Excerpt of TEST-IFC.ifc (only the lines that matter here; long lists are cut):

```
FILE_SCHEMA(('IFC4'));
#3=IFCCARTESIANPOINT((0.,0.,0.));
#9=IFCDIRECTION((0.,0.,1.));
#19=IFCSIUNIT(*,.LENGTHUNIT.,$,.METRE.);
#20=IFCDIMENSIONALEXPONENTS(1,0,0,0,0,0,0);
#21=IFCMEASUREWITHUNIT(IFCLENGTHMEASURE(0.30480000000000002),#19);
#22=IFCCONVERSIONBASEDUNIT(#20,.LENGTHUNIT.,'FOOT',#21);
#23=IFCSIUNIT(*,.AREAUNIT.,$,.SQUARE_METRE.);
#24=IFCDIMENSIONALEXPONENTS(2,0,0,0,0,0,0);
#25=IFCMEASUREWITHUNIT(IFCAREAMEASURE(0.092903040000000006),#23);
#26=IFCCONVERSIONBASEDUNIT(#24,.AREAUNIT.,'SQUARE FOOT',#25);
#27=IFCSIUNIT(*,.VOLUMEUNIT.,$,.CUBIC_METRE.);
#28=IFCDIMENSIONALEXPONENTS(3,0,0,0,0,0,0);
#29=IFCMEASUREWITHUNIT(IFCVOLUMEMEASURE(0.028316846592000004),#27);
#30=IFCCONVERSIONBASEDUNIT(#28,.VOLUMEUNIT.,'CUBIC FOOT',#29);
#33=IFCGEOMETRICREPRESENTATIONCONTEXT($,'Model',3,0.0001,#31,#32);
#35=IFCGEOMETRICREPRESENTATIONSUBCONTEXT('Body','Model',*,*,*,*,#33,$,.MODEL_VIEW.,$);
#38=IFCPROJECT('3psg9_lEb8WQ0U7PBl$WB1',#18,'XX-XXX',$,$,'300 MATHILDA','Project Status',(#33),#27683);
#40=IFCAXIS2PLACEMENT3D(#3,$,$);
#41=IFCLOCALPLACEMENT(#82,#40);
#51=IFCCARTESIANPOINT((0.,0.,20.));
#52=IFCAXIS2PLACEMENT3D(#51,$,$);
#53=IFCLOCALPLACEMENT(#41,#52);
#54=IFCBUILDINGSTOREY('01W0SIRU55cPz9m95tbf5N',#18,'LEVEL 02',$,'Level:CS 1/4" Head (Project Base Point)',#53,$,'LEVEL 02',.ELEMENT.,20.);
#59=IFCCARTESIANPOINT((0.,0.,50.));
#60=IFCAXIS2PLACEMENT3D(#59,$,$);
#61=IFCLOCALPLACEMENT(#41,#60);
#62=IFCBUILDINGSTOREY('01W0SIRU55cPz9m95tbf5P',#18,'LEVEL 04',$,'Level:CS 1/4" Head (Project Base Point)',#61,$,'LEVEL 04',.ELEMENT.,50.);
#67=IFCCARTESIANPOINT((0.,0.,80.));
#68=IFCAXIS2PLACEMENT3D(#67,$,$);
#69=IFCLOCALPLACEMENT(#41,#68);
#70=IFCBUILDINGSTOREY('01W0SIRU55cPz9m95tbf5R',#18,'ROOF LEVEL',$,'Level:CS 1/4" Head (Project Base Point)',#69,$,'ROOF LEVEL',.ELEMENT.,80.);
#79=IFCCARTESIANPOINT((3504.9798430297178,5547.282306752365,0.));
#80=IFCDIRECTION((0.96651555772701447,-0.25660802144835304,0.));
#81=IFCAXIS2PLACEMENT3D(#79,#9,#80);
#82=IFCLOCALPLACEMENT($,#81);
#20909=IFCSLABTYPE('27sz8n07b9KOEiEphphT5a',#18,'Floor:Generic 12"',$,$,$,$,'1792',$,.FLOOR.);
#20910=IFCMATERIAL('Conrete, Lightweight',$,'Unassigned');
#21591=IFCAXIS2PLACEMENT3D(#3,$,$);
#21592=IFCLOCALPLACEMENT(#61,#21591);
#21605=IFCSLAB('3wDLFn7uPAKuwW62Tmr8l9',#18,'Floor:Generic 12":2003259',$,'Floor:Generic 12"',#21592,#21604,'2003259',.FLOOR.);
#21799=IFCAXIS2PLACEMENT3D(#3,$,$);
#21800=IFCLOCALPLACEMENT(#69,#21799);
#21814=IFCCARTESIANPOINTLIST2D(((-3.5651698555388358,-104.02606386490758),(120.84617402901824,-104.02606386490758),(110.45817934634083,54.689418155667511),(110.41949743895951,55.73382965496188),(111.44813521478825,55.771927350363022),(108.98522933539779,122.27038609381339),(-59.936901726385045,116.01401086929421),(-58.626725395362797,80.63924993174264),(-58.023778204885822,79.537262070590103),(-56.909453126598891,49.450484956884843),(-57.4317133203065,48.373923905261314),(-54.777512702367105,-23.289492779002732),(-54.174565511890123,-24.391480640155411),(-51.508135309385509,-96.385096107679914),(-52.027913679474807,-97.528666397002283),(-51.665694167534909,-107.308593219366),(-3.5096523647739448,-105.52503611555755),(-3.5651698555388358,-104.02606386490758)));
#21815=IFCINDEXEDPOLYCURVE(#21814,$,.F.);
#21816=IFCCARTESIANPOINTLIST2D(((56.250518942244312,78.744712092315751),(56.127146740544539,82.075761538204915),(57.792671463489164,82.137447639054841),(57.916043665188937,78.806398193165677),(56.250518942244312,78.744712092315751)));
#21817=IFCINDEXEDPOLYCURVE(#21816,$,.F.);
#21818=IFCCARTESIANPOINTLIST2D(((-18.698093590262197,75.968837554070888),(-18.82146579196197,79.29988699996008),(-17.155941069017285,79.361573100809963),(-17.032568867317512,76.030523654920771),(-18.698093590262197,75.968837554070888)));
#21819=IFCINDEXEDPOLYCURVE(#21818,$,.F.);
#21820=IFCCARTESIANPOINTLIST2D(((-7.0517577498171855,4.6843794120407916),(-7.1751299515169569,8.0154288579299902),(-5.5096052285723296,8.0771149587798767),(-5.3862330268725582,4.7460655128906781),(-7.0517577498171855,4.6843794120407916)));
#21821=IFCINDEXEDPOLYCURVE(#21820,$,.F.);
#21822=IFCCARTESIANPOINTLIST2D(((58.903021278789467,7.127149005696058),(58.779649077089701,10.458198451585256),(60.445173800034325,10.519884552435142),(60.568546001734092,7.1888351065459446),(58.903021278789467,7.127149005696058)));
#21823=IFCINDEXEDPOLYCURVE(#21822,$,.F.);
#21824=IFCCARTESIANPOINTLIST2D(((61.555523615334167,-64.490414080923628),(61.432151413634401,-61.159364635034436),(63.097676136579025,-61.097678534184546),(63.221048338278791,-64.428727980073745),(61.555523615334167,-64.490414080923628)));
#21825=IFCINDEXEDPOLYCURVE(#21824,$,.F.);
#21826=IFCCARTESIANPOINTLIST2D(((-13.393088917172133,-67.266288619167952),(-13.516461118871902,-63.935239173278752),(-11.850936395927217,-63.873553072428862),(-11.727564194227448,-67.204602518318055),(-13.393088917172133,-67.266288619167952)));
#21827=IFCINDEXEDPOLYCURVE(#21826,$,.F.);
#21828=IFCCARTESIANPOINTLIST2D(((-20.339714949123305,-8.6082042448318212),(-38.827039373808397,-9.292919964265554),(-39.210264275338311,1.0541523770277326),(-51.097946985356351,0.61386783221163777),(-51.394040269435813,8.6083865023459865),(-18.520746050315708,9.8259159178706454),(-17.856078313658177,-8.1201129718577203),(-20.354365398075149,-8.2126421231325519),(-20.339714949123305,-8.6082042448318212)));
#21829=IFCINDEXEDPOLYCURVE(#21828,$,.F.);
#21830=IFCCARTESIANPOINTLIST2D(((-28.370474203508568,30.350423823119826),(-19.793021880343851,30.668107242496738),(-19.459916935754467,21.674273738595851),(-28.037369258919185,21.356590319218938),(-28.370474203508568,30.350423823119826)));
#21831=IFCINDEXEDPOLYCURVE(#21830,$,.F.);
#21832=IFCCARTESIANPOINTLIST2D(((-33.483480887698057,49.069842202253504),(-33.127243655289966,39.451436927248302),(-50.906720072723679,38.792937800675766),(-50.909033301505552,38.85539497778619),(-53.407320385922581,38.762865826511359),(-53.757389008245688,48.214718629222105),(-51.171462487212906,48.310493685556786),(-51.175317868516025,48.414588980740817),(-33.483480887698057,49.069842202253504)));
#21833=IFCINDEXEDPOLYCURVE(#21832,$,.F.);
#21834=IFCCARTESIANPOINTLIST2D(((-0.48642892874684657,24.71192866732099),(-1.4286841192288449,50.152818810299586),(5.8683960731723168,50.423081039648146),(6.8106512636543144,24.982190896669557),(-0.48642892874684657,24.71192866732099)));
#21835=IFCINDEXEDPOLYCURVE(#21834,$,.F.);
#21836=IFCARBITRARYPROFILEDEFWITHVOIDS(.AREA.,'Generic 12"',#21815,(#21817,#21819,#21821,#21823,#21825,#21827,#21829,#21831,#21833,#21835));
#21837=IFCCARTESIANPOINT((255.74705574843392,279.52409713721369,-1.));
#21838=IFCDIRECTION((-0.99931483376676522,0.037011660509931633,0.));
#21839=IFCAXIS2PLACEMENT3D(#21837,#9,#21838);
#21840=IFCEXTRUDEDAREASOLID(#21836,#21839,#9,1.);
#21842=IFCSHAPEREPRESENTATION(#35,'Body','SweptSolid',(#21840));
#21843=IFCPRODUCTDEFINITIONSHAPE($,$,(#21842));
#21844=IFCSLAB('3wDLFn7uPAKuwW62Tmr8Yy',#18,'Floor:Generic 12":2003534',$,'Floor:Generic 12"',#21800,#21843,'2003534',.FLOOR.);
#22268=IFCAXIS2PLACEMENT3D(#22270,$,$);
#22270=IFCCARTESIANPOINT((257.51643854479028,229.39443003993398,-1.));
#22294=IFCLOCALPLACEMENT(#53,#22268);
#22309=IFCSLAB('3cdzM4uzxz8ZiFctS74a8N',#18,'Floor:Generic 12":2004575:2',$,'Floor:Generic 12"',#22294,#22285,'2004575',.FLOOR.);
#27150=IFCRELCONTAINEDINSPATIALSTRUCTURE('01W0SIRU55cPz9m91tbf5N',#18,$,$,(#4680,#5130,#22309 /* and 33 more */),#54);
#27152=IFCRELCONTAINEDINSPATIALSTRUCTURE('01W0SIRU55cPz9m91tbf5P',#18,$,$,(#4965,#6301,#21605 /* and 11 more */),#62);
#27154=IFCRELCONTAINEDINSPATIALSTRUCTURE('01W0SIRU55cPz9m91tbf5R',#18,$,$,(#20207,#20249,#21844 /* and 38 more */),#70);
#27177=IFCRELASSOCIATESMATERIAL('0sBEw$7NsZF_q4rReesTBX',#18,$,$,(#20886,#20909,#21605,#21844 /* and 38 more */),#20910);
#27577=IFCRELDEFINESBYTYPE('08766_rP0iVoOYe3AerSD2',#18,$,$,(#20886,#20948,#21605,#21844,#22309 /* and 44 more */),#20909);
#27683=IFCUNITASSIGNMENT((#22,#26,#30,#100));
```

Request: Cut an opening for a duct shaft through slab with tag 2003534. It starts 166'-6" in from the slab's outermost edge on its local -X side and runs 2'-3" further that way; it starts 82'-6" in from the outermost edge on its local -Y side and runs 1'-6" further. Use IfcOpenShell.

```python
import numpy as np
import ifcopenshell
import ifcopenshell.api.feature
import ifcopenshell.api.geometry
import ifcopenshell.api.root
import ifcopenshell.geom
import ifcopenshell.util.placement
import ifcopenshell.util.representation
import ifcopenshell.util.shape
import ifcopenshell.util.unit

model = ifcopenshell.open("TEST-IFC.ifc")
unit_scale = ifcopenshell.util.unit.calculate_unit_scale(model)
settings = ifcopenshell.geom.settings()


def volume(element):
    """Net volume in cubic metres, openings subtracted."""
    shape = ifcopenshell.geom.create_shape(settings, element)
    return ifcopenshell.util.shape.get_volume(shape.geometry)


slab = model.by_guid("3wDLFn7uPAKuwW62Tmr8Yy")
before = volume(slab)

# Extent in the slab's own axes, in metres. The edges named are its -X and -Y sides.
slab_shape = ifcopenshell.geom.create_shape(settings, slab)
vertices = ifcopenshell.util.shape.get_vertices(slab_shape.geometry)
x_min, y_min, bottom = vertices.min(axis=0)
top = vertices[:, 2].max()

opening = ifcopenshell.api.root.create_entity(model, ifc_class="IfcOpeningElement", name="Duct shaft opening", predefined_type="OPENING")
context = ifcopenshell.util.representation.get_context(model, "Model", "Body", "MODEL_VIEW")
width, depth = 0.6858, 0.4572
outline = [(0.0, 0.0), (width, 0.0), (width, depth), (0.0, depth), (0.0, 0.0)]
# Overshoot both faces by 50 mm so the cut is clean.
shape = ifcopenshell.api.geometry.add_slab_representation(
    model, context=context, depth=top - bottom + 0.1, polyline=outline
)
ifcopenshell.api.geometry.assign_representation(model, product=opening, representation=shape)

matrix = ifcopenshell.util.placement.get_local_placement(slab.ObjectPlacement)
matrix[:, 3] = matrix @ np.append(np.array([x_min + 50.7492, y_min + 25.146, bottom - 0.05]) / unit_scale, 1.0)
ifcopenshell.api.geometry.edit_object_placement(model, product=opening, matrix=matrix, is_si=False)
ifcopenshell.api.feature.add_feature(model, feature=opening, element=slab)

after = volume(slab)

print(f"slab volume {before:.3f} -> {after:.3f} m3")

model.write("TEST-IFC_edited.ifc")
```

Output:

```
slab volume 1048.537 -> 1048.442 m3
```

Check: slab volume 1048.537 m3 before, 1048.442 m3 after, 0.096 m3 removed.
